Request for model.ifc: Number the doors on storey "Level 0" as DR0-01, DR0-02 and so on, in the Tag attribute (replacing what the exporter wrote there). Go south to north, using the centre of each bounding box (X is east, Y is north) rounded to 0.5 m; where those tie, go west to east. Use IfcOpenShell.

First a look at what the model holds.

```python
import ifcopenshell
import ifcopenshell.util.element
import ifcopenshell.util.placement

model = ifcopenshell.open("model.ifc")
print(model.schema)
storey = next(s for s in model.by_type("IfcBuildingStorey") if s.Name == "Level 0")
doors = [e for e in ifcopenshell.util.element.get_decomposition(storey) if e.is_a("IfcDoor")]
for e in sorted(doors, key=lambda e: e.id()):
    origin = ifcopenshell.util.placement.get_local_placement(e.ObjectPlacement)[:3, 3]
    print(e.id(), e.Tag, e.Name, origin.round(2) + 0.0, sep=" | ")
```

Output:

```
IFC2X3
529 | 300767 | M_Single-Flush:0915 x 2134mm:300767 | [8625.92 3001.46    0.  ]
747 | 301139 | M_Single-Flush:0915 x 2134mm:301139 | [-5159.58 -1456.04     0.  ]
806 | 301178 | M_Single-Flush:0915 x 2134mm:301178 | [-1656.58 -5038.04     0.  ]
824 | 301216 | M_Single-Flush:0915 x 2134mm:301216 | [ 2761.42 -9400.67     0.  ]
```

```python
import ifcopenshell
import ifcopenshell.geom
import ifcopenshell.util.element
import ifcopenshell.util.shape

model = ifcopenshell.open("model.ifc")
settings = ifcopenshell.geom.settings()
settings.set("use-world-coords", True)


def centre(element):
    shape = ifcopenshell.geom.create_shape(settings, element)
    return ifcopenshell.util.shape.get_bbox_centroid(shape.geometry)


storey = next(s for s in model.by_type("IfcBuildingStorey") if s.Name == "Level 0")
doors = [e for e in ifcopenshell.util.element.get_decomposition(storey) if e.is_a("IfcDoor")]

# Insertion points can sit at a corner or the storey origin, so sort by the geometry (in metres).
centres = {e: centre(e) for e in doors}
doors.sort(key=lambda e: (round(centres[e][1] / 0.5), centres[e][0]))

for i, e in enumerate(doors, start=1):
    number = f"DR0-{i:02d}"
    e.Tag = number
    print(e.id(), number)

model.write("model_v2.ifc")
```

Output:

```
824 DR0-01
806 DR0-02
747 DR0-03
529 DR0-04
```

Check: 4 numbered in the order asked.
